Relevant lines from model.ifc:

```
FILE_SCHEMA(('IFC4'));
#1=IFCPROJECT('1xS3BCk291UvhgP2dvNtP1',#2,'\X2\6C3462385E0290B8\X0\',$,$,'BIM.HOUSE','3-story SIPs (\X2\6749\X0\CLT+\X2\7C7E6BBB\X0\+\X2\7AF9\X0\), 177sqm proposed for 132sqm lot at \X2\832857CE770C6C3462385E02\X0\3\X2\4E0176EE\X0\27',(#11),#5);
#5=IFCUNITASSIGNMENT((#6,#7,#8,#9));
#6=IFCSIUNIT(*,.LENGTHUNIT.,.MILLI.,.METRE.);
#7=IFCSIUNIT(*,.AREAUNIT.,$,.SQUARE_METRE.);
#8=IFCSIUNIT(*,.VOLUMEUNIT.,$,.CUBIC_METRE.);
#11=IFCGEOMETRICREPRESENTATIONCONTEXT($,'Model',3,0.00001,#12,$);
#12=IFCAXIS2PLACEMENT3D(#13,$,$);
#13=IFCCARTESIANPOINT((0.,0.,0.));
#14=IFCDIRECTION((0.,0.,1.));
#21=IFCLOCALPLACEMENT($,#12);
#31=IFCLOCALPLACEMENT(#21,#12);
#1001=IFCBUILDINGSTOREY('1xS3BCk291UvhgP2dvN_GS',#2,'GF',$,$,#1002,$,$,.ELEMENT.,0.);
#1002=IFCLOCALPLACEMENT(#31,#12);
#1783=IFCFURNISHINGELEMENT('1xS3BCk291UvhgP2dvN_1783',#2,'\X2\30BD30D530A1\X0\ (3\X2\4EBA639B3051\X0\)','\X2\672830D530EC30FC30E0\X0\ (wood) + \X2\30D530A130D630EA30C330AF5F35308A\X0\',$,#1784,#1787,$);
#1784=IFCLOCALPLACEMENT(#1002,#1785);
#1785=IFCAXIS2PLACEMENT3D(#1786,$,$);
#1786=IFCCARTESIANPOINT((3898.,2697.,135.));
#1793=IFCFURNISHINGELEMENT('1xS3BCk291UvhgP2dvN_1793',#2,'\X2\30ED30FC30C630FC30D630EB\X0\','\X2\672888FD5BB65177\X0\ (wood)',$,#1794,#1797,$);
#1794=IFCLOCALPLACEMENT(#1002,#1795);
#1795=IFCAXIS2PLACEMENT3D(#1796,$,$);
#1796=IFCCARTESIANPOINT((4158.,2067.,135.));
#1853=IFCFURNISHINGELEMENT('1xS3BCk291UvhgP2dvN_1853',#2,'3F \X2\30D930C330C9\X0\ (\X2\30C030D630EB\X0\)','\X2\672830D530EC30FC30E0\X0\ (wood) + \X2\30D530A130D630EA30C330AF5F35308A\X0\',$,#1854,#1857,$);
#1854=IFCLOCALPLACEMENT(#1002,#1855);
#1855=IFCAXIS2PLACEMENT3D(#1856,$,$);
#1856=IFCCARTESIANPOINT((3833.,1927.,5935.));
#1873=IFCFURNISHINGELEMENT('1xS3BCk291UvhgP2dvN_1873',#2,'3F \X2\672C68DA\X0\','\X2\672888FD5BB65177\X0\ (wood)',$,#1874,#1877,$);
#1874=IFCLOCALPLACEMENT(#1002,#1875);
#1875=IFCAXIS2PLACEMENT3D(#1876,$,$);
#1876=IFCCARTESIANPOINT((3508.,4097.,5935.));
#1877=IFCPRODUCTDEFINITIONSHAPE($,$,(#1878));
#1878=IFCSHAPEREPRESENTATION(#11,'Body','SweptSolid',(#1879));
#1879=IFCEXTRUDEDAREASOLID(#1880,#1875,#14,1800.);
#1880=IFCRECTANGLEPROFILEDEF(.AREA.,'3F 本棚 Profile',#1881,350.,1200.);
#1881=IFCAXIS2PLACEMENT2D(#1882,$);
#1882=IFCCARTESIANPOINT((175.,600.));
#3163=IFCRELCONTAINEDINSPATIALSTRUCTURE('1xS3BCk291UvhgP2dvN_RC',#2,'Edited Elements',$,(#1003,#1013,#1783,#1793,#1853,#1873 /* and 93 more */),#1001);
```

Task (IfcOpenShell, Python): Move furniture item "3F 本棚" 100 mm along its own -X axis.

```python
import ifcopenshell
import ifcopenshell.api.geometry
import ifcopenshell.util.placement
import ifcopenshell.util.unit

model = ifcopenshell.open("model.ifc")
unit_scale = ifcopenshell.util.unit.calculate_unit_scale(model)

item = model.by_guid("1xS3BCk291UvhgP2dvN_1873")
matrix = ifcopenshell.util.placement.get_local_placement(item.ObjectPlacement)
matrix[:3, 3] -= matrix[:3, 0] * 0.1 / unit_scale
ifcopenshell.api.geometry.edit_object_placement(model, product=item, matrix=matrix, is_si=False)

print(ifcopenshell.util.placement.get_local_placement(item.ObjectPlacement).round(3) + 0.0)

model.write("model_edited.ifc")
```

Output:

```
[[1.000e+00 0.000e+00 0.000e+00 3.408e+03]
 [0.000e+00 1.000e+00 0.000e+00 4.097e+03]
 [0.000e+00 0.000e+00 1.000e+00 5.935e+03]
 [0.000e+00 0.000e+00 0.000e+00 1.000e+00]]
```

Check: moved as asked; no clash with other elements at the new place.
